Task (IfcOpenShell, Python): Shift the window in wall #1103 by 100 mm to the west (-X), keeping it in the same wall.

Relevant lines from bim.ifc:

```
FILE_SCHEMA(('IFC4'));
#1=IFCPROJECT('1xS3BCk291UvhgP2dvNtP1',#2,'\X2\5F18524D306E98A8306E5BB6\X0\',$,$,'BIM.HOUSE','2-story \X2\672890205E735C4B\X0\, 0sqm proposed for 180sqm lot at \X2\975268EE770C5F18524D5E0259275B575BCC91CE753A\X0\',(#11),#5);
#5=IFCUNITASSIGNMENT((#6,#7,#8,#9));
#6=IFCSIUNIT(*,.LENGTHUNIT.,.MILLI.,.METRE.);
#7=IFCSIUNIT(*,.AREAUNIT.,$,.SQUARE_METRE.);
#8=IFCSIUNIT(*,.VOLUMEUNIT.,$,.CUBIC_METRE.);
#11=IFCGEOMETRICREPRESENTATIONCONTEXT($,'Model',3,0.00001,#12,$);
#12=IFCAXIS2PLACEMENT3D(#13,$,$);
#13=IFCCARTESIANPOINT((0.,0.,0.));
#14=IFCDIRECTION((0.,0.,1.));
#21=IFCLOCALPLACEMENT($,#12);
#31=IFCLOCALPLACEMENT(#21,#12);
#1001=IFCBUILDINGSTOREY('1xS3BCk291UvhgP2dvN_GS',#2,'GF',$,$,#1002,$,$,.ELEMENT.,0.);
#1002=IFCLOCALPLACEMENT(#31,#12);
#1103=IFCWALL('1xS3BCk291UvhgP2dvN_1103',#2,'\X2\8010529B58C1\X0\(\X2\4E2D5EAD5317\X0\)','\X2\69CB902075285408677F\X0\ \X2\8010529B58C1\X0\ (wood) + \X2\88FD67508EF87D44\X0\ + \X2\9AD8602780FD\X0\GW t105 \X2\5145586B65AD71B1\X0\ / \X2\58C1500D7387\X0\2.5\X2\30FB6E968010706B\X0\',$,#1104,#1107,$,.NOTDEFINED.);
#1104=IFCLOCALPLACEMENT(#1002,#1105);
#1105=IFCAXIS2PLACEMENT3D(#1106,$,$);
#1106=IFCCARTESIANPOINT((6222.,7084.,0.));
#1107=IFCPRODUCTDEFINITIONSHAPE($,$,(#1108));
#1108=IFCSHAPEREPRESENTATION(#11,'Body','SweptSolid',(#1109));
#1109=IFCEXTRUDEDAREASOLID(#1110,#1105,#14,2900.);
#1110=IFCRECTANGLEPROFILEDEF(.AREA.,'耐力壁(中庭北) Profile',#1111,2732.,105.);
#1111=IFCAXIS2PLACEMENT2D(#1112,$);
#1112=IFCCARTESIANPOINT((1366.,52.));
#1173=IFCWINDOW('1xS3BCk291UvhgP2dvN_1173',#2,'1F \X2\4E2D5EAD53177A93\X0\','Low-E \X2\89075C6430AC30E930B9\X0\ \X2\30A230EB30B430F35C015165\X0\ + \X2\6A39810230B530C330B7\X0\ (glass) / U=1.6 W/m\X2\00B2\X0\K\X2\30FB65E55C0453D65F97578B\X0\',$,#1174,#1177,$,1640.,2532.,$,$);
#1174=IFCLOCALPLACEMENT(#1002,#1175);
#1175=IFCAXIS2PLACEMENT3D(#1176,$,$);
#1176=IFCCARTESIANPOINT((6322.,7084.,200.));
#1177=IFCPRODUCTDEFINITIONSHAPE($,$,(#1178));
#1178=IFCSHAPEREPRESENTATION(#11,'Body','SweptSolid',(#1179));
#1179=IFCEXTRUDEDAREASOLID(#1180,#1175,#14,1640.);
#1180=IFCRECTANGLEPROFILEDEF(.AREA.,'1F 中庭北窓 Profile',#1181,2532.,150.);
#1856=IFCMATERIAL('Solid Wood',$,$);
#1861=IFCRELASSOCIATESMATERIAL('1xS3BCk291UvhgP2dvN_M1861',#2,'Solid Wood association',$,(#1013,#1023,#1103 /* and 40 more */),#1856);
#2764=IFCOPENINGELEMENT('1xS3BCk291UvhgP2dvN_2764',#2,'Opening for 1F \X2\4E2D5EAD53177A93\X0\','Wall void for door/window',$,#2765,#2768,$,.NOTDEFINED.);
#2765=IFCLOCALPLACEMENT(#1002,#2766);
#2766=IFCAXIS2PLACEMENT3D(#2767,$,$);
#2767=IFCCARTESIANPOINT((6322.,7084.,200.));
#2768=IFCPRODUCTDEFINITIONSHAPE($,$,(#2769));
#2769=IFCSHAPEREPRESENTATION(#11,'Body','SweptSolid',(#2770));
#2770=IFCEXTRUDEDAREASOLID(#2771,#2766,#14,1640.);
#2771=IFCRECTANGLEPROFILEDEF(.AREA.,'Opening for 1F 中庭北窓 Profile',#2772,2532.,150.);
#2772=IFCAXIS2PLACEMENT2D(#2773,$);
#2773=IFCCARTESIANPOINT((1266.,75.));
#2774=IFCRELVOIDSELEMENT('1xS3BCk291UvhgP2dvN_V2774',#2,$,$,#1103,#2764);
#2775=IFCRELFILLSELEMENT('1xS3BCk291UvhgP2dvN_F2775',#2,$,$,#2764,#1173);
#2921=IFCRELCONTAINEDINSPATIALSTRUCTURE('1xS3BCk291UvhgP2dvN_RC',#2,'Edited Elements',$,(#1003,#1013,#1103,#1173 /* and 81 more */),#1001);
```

```python
import ifcopenshell
import ifcopenshell.api.geometry
import ifcopenshell.util.placement
import ifcopenshell.util.unit

model = ifcopenshell.open("bim.ifc")
unit_scale = ifcopenshell.util.unit.calculate_unit_scale(model)

window = model.by_id(1173)
opening = window.FillsVoids[0].RelatingOpeningElement
wall = opening.VoidsElements[0].RelatingBuildingElement

wall_matrix = ifcopenshell.util.placement.get_local_placement(wall.ObjectPlacement)
shift = wall_matrix[:3, 0] * -0.1 / unit_scale
before = ifcopenshell.util.placement.get_local_placement(window.ObjectPlacement)[:3, 3].copy()

# The window is not placed relative to its opening, so move both.
for product in (opening, window):
    matrix = ifcopenshell.util.placement.get_local_placement(product.ObjectPlacement)
    matrix[:3, 3] += shift
    ifcopenshell.api.geometry.edit_object_placement(model, product=product, matrix=matrix, is_si=False)

after = ifcopenshell.util.placement.get_local_placement(window.ObjectPlacement)[:3, 3]
print("window moved by", (after - before).round(3) + 0.0)

model.write("bim-out.ifc")
```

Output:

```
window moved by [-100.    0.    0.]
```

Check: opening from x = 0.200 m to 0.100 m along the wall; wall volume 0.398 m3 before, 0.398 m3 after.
